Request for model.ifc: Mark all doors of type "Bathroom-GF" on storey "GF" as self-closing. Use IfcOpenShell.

First a look at what the model holds.

```python
import ifcopenshell
import ifcopenshell.util.element

model = ifcopenshell.open("model.ifc")
print(model.schema)
storey = next(s for s in model.by_type("IfcBuildingStorey") if s.Name == "GF")
doors = [e for e in ifcopenshell.util.element.get_decomposition(storey) if e.is_a("IfcDoor")]
seen = {}
for e in doors:
    element_type = ifcopenshell.util.element.get_type(e)
    key = (element_type.Name if element_type != e and element_type else None, ifcopenshell.util.element.get_pset(e, "Pset_DoorCommon", "SelfClosing"))
    seen[key] = seen.get(key, 0) + 1
for (name, value), count in sorted(seen.items(), key=str):
    print(count, "x", name, "|", value)
```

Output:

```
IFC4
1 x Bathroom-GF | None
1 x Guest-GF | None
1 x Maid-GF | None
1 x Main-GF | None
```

```python
import ifcopenshell
import ifcopenshell.api.pset
import ifcopenshell.util.element

model = ifcopenshell.open("model.ifc")

storey = next(s for s in model.by_type("IfcBuildingStorey") if s.Name == "GF")
doors = [e for e in ifcopenshell.util.element.get_decomposition(storey) if e.is_a("IfcDoor")]

count = 0
for e in doors:
    element_type = ifcopenshell.util.element.get_type(e)
    if element_type in (None, e) or element_type.Name != "Bathroom-GF":
        continue
    # add_pset returns the element's existing set when there is one.
    pset = ifcopenshell.api.pset.add_pset(model, product=e, name="Pset_DoorCommon")
    ifcopenshell.api.pset.edit_pset(model, pset=pset, properties={"SelfClosing": True})
    count += 1

print(count, "doors updated")

model.write("model-out.ifc")
```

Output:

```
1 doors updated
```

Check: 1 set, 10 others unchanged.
